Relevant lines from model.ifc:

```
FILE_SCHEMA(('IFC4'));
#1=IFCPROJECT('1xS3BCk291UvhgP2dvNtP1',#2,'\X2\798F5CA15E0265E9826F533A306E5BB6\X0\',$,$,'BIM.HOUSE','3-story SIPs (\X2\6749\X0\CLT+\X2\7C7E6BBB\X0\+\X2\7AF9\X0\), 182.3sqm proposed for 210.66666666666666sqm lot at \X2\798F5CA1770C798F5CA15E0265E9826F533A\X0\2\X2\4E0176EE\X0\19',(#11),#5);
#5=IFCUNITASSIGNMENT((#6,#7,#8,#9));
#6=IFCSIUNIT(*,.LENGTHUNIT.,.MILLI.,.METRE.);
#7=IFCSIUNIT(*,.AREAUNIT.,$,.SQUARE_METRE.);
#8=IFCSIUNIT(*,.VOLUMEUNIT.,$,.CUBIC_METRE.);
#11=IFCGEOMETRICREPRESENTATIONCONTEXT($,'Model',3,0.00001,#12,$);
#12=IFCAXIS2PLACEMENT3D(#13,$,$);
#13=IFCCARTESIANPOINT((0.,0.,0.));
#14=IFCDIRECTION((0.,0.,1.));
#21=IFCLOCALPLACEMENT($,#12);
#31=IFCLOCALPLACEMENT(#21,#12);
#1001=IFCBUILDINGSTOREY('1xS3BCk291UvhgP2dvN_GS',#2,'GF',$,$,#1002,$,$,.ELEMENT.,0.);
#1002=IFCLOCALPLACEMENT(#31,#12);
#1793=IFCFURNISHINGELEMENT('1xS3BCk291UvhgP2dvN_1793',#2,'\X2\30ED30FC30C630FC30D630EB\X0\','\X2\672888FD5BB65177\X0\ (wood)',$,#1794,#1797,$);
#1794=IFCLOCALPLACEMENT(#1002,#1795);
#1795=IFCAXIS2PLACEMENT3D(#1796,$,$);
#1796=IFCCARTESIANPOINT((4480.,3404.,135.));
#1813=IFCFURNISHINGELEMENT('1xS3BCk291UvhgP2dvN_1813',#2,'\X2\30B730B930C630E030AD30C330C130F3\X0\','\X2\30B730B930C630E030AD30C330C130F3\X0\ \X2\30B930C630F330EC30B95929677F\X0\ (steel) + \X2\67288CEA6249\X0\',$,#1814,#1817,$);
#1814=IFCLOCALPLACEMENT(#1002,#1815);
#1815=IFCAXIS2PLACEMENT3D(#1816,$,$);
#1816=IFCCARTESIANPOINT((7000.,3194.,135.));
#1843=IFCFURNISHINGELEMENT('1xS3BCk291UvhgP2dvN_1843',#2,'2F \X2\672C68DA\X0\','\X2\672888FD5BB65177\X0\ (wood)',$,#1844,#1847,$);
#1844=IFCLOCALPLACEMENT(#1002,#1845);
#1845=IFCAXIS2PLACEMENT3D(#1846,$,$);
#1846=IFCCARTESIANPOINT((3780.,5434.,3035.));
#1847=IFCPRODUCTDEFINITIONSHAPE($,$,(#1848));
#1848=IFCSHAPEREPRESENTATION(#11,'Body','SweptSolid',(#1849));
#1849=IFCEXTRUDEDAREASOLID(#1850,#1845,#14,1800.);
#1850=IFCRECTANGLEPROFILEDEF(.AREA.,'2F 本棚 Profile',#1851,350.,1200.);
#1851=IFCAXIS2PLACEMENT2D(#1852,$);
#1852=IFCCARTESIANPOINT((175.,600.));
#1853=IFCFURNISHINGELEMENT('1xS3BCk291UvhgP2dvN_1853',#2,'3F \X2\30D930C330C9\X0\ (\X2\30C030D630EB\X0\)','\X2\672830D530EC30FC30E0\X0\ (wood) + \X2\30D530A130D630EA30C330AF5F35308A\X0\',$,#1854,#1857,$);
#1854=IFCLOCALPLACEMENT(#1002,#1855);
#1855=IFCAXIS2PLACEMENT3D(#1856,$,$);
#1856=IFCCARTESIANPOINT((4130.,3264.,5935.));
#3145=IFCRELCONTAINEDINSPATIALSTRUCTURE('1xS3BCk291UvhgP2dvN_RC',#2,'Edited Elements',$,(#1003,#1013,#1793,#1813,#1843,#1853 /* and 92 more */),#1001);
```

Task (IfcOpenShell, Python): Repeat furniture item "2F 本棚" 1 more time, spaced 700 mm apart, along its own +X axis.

```python
import ifcopenshell
import ifcopenshell.api.geometry
import ifcopenshell.api.root
import ifcopenshell.util.element
import ifcopenshell.util.placement
import ifcopenshell.util.unit

model = ifcopenshell.open("model.ifc")
unit_scale = ifcopenshell.util.unit.calculate_unit_scale(model)


def reuse_history(source, copy):
    """copy_class also copies each property set's owner history, people and application; keep the originals."""
    for rel in copy.IsDefinedBy:
        if rel.is_a("IfcRelDefinesByProperties") and (history := rel.RelatingPropertyDefinition.OwnerHistory):
            rel.RelatingPropertyDefinition.OwnerHistory = source.OwnerHistory
            ifcopenshell.util.element.remove_deep2(model, history)


source = model.by_guid("1xS3BCk291UvhgP2dvN_1843")
base = ifcopenshell.util.placement.get_local_placement(source.ObjectPlacement)
step = base[:3, 0] * 0.7 / unit_scale

for i in range(1, 2):
    copy = ifcopenshell.api.root.copy_class(model, product=source)
    copy.Representation = ifcopenshell.util.element.copy_deep(
        model, source.Representation, exclude=["IfcGeometricRepresentationContext", "IfcRepresentationMap"]
    )
    reuse_history(source, copy)
    matrix = base.copy()
    matrix[:3, 3] += i * step
    print("added at", matrix[:3, 3].round(3) + 0.0)
    ifcopenshell.api.geometry.edit_object_placement(model, product=copy, matrix=matrix, is_si=False)

model.write("model_rev.ifc")
```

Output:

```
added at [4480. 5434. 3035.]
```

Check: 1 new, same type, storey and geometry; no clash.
